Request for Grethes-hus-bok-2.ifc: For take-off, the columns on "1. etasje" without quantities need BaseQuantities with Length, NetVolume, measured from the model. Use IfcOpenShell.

First a look at what the model holds.

```python
import ifcopenshell
import ifcopenshell.util.element
import ifcopenshell.util.unit

model = ifcopenshell.open("Grethes-hus-bok-2.ifc")
print(model.schema)
for unit_type in ("LENGTHUNIT", "AREAUNIT", "VOLUMEUNIT"):
    print(unit_type, ifcopenshell.util.unit.calculate_unit_scale(model, unit_type))
storey = next(s for s in model.by_type("IfcBuildingStorey") if s.Name == "1. etasje")
columns = [e for e in ifcopenshell.util.element.get_decomposition(storey) if e.is_a("IfcColumn")]
for e in sorted(columns, key=lambda e: e.id()):
    print(e.id(), e.is_a(), e.Name, list(ifcopenshell.util.element.get_psets(e, qtos_only=True)), sep=" | ")
```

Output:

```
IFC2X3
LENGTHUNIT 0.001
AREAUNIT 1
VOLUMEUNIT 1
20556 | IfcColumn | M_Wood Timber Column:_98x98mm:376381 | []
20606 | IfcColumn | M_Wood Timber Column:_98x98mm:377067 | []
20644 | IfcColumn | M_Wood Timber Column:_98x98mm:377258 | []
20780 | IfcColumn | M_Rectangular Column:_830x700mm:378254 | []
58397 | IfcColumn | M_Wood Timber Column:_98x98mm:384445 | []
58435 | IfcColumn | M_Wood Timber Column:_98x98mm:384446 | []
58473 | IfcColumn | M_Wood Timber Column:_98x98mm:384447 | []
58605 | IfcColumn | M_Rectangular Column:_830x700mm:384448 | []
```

```python
import ifcopenshell
import ifcopenshell.api.pset
import ifcopenshell.geom
import ifcopenshell.util.element
import ifcopenshell.util.shape
import ifcopenshell.util.unit

model = ifcopenshell.open("Grethes-hus-bok-2.ifc")
unit_scale = ifcopenshell.util.unit.calculate_unit_scale(model)
volume_scale = ifcopenshell.util.unit.calculate_unit_scale(model, "VOLUMEUNIT")
settings = ifcopenshell.geom.settings()

storey = next(s for s in model.by_type("IfcBuildingStorey") if s.Name == "1. etasje")
columns = [e for e in ifcopenshell.util.element.get_decomposition(storey) if e.is_a("IfcColumn")]

for e in sorted(columns, key=lambda e: e.id()):
    if ifcopenshell.util.element.get_psets(e, qtos_only=True, should_inherit=False):
        continue
    # Geometry comes back in metres, in the element's own axes.
    shape = ifcopenshell.geom.create_shape(settings, e)
    values = {
        "Length": ifcopenshell.util.shape.get_z(shape.geometry) / unit_scale,
        "NetVolume": ifcopenshell.util.shape.get_volume(shape.geometry) / volume_scale,
    }
    qto = ifcopenshell.api.pset.add_qto(model, product=e, name="BaseQuantities")
    ifcopenshell.api.pset.edit_qto(model, qto=qto, properties=values)
    print(e.id(), {k: round(v, 3) for k, v in values.items()})

model.write("Grethes-hus-bok-2-out.ifc")
```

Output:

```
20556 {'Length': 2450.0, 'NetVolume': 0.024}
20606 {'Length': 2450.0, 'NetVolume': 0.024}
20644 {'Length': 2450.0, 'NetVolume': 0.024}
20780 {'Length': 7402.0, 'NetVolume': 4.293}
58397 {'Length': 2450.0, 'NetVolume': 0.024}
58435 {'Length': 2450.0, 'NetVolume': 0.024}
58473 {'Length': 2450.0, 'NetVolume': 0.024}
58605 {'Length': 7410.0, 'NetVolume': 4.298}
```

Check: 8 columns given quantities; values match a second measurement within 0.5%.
